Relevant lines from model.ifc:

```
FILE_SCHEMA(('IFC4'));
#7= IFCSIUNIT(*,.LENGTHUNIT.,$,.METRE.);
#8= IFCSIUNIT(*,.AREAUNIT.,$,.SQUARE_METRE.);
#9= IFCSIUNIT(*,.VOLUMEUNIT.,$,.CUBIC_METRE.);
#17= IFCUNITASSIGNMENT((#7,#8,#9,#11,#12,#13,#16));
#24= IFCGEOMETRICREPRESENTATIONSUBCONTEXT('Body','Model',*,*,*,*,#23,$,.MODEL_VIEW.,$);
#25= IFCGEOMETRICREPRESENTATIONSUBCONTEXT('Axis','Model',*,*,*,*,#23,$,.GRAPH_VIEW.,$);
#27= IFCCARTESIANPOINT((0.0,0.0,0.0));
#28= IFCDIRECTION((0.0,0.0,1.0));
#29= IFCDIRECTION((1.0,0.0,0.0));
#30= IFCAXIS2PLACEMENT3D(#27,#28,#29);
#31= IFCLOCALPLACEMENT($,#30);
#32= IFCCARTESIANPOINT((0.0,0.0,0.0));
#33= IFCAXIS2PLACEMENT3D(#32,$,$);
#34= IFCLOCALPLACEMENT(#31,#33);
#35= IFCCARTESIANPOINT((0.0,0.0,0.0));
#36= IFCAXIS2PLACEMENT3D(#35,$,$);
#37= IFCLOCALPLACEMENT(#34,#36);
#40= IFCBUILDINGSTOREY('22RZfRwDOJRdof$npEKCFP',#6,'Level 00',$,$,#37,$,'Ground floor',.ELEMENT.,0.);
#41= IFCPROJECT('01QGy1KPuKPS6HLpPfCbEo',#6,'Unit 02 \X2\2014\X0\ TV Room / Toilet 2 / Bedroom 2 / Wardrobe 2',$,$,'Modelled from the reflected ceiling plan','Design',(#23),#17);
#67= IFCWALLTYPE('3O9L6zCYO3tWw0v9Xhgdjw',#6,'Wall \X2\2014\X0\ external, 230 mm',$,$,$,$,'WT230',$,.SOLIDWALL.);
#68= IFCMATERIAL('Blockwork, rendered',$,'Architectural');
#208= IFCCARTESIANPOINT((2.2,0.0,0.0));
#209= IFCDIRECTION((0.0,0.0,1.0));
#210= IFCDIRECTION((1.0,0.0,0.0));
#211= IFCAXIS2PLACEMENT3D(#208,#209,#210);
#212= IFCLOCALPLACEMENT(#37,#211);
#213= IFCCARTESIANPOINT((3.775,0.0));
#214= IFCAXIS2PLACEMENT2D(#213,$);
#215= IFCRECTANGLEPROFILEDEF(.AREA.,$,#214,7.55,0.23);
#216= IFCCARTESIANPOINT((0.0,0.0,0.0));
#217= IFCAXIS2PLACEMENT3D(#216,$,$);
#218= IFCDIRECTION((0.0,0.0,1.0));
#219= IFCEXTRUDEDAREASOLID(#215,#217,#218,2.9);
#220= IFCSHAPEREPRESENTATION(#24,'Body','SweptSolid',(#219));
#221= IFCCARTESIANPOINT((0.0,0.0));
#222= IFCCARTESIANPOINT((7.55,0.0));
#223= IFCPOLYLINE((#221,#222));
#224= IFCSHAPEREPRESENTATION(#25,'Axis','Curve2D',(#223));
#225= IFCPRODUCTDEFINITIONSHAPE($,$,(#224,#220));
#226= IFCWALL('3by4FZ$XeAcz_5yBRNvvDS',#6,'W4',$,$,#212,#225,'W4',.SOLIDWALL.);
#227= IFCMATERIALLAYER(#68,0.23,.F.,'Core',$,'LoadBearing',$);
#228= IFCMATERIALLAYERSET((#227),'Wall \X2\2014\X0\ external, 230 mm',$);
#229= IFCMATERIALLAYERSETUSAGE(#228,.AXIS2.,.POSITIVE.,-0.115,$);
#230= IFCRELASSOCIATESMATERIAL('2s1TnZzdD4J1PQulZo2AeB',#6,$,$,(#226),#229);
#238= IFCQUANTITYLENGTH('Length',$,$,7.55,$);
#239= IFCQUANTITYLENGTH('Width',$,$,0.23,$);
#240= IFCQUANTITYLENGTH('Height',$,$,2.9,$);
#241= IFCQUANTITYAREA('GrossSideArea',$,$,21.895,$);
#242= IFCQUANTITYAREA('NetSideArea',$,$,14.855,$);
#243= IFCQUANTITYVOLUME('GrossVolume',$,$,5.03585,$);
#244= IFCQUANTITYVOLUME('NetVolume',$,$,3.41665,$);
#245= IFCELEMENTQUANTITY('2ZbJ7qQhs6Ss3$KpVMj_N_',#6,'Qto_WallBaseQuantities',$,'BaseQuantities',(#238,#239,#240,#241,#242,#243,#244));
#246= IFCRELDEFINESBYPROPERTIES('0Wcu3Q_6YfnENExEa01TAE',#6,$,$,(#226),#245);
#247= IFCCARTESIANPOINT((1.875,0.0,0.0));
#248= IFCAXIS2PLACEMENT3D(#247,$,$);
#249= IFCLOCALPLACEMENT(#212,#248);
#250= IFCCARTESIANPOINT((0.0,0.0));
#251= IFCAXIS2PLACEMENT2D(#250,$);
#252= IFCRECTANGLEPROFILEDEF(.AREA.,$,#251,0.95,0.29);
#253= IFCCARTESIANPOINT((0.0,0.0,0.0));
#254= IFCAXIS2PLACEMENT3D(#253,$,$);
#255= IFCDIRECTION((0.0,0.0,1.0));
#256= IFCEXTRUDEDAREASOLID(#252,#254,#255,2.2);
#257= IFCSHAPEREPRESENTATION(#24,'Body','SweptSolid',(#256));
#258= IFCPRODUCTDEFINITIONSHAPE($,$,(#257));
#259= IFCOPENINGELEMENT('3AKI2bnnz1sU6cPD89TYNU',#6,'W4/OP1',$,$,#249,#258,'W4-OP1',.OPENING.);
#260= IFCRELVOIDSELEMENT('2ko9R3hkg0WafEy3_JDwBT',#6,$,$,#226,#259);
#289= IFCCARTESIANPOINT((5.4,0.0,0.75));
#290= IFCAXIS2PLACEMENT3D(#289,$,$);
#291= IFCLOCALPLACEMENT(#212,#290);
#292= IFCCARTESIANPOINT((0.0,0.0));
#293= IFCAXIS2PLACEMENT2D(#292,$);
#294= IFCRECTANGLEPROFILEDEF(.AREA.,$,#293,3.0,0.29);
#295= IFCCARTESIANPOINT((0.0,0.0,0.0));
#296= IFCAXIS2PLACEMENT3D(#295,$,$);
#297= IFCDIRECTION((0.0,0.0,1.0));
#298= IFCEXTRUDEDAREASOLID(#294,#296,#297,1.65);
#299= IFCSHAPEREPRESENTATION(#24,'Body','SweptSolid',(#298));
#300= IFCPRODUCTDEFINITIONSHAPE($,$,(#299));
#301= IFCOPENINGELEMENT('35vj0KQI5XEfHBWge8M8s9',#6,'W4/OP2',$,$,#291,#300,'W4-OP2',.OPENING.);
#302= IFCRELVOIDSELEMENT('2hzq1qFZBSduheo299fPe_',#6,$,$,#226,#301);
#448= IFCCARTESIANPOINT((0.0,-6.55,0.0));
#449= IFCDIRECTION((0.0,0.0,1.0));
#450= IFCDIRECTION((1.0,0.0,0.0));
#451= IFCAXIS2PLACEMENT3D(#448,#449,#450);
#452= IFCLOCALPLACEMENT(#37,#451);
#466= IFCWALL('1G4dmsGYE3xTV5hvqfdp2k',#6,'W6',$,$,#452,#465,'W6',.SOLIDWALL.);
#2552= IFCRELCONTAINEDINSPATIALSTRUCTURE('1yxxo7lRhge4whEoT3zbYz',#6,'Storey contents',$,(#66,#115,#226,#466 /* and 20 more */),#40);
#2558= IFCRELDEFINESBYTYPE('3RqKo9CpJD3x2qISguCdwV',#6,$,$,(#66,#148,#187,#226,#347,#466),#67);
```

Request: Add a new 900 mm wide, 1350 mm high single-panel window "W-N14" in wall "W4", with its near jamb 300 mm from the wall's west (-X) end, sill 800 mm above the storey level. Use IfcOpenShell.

```python
import numpy as np
import ifcopenshell
import ifcopenshell.api.feature
import ifcopenshell.api.geometry
import ifcopenshell.api.pset
import ifcopenshell.api.root
import ifcopenshell.api.spatial
import ifcopenshell.geom
import ifcopenshell.util.element
import ifcopenshell.util.placement
import ifcopenshell.util.representation
import ifcopenshell.util.shape
import ifcopenshell.util.unit

model = ifcopenshell.open("model.ifc")
unit_scale = ifcopenshell.util.unit.calculate_unit_scale(model)
area_scale = ifcopenshell.util.unit.calculate_unit_scale(model, "AREAUNIT")
volume_scale = ifcopenshell.util.unit.calculate_unit_scale(model, "VOLUMEUNIT")
settings = ifcopenshell.geom.settings()


def volume(element):
    """Net volume in cubic metres, openings subtracted."""
    shape = ifcopenshell.geom.create_shape(settings, element)
    return ifcopenshell.util.shape.get_volume(shape.geometry)


wall = model.by_guid("3by4FZ$XeAcz_5yBRNvvDS")
storey = ifcopenshell.util.element.get_container(wall, ifc_class="IfcBuildingStorey")
context = ifcopenshell.util.representation.get_context(model, "Model", "Body", "MODEL_VIEW")
before = volume(wall)

width, height, from_end, sill = 0.9, 1.35, 0.3, 0.8  # metres

# The wall runs along its own X axis, and the end named is its -X end.
wall_shape = ifcopenshell.geom.create_shape(settings, wall)
x, y, z = ifcopenshell.util.shape.get_vertices(wall_shape.geometry).T
start = x.min() + from_end
face, thickness = float(y.min()), float(y.max() - y.min())
wall_matrix = ifcopenshell.util.placement.get_local_placement(wall.ObjectPlacement)
level = ifcopenshell.util.placement.get_local_placement(storey.ObjectPlacement)[2, 3]


def in_wall(x, y):
    """Placement at x, y metres in the wall's axes, at sill height."""
    matrix = wall_matrix.copy()
    matrix[:, 3] = wall_matrix @ np.array([x / unit_scale, y / unit_scale, 0.0, 1.0])
    matrix[2, 3] = level + sill / unit_scale
    return matrix


# Opening: a box that overshoots both wall faces by 50 mm.
opening = ifcopenshell.api.root.create_entity(model, ifc_class="IfcOpeningElement", predefined_type="OPENING")
box = ifcopenshell.api.geometry.add_wall_representation(
    model, context=context, length=width, height=height, thickness=thickness + 0.1
)
ifcopenshell.api.geometry.assign_representation(model, product=opening, representation=box)
ifcopenshell.api.geometry.edit_object_placement(model, product=opening, matrix=in_wall(start, face - 0.05), is_si=False)
ifcopenshell.api.feature.add_feature(model, feature=opening, element=wall)

window = ifcopenshell.api.root.create_entity(model, ifc_class="IfcWindow", name="W-N14", predefined_type="WINDOW")
window.OverallWidth, window.OverallHeight = width / unit_scale, height / unit_scale
window.PartitioningType = "SINGLE_PANEL"
body = ifcopenshell.api.geometry.add_window_representation(
    model,
    context=context,
    overall_width=window.OverallWidth,
    overall_height=window.OverallHeight,
    partition_type="SINGLE_PANEL",
)
ifcopenshell.api.geometry.assign_representation(model, product=window, representation=body)
ifcopenshell.api.spatial.assign_container(model, products=[window], relating_structure=storey)
ifcopenshell.api.feature.add_filling(model, opening=opening, element=window)

# Centre the window in the wall's thickness.
ifcopenshell.api.geometry.edit_object_placement(model, product=window, matrix=in_wall(start, face), is_si=False)
window_shape = ifcopenshell.geom.create_shape(settings, window)
depth = ifcopenshell.util.shape.get_vertices(window_shape.geometry)[:, 1]
offset = face + thickness / 2 - (depth.min() + depth.max()) / 2
ifcopenshell.api.geometry.edit_object_placement(model, product=window, matrix=in_wall(start, offset), is_si=False)

after = volume(wall)

# Update the wall's stored quantities.
qto = model.by_id(ifcopenshell.util.element.get_pset(wall, "Qto_WallBaseQuantities", should_inherit=False)["id"])
ifcopenshell.api.pset.edit_qto(model, qto=qto, properties={
    "NetSideArea": after / thickness / area_scale,
    "NetVolume": after / volume_scale,
})

print(f"wall volume {before:.3f} -> {after:.3f} m3")

model.write("model_v2.ifc")
```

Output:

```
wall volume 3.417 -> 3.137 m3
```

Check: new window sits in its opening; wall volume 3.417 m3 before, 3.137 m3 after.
